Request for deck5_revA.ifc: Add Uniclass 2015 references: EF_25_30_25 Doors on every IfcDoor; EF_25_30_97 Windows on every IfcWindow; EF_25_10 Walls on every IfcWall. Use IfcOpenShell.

First a look at what the model holds.

```python
import ifcopenshell

model = ifcopenshell.open("deck5_revA.ifc")
print(model.schema)
print("classifications:", [c.Name for c in model.by_type("IfcClassification")])
for ifc_class in ("IfcDoor", "IfcRoof", "IfcStair", "IfcWall", "IfcWindow"):
    print(ifc_class, len(model.by_type(ifc_class)))
```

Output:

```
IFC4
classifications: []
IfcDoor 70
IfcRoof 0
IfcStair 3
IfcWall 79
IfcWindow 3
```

```python
import ifcopenshell
import ifcopenshell.api.classification

model = ifcopenshell.open("deck5_revA.ifc")

system = ifcopenshell.api.classification.add_classification(model, classification="Uniclass 2015")

codes = {
    "IfcDoor": ("EF_25_30_25", "Doors"),
    "IfcWindow": ("EF_25_30_97", "Windows"),
    "IfcWall": ("EF_25_10", "Walls"),
}
for ifc_class, (code, name) in codes.items():
    products = model.by_type(ifc_class)
    ifcopenshell.api.classification.add_reference(
        model, products=products, classification=system, identification=code, name=name
    )
    print(code, len(products))

model.write("deck5_revA-out.ifc")
```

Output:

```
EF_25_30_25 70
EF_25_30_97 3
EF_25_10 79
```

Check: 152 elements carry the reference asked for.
